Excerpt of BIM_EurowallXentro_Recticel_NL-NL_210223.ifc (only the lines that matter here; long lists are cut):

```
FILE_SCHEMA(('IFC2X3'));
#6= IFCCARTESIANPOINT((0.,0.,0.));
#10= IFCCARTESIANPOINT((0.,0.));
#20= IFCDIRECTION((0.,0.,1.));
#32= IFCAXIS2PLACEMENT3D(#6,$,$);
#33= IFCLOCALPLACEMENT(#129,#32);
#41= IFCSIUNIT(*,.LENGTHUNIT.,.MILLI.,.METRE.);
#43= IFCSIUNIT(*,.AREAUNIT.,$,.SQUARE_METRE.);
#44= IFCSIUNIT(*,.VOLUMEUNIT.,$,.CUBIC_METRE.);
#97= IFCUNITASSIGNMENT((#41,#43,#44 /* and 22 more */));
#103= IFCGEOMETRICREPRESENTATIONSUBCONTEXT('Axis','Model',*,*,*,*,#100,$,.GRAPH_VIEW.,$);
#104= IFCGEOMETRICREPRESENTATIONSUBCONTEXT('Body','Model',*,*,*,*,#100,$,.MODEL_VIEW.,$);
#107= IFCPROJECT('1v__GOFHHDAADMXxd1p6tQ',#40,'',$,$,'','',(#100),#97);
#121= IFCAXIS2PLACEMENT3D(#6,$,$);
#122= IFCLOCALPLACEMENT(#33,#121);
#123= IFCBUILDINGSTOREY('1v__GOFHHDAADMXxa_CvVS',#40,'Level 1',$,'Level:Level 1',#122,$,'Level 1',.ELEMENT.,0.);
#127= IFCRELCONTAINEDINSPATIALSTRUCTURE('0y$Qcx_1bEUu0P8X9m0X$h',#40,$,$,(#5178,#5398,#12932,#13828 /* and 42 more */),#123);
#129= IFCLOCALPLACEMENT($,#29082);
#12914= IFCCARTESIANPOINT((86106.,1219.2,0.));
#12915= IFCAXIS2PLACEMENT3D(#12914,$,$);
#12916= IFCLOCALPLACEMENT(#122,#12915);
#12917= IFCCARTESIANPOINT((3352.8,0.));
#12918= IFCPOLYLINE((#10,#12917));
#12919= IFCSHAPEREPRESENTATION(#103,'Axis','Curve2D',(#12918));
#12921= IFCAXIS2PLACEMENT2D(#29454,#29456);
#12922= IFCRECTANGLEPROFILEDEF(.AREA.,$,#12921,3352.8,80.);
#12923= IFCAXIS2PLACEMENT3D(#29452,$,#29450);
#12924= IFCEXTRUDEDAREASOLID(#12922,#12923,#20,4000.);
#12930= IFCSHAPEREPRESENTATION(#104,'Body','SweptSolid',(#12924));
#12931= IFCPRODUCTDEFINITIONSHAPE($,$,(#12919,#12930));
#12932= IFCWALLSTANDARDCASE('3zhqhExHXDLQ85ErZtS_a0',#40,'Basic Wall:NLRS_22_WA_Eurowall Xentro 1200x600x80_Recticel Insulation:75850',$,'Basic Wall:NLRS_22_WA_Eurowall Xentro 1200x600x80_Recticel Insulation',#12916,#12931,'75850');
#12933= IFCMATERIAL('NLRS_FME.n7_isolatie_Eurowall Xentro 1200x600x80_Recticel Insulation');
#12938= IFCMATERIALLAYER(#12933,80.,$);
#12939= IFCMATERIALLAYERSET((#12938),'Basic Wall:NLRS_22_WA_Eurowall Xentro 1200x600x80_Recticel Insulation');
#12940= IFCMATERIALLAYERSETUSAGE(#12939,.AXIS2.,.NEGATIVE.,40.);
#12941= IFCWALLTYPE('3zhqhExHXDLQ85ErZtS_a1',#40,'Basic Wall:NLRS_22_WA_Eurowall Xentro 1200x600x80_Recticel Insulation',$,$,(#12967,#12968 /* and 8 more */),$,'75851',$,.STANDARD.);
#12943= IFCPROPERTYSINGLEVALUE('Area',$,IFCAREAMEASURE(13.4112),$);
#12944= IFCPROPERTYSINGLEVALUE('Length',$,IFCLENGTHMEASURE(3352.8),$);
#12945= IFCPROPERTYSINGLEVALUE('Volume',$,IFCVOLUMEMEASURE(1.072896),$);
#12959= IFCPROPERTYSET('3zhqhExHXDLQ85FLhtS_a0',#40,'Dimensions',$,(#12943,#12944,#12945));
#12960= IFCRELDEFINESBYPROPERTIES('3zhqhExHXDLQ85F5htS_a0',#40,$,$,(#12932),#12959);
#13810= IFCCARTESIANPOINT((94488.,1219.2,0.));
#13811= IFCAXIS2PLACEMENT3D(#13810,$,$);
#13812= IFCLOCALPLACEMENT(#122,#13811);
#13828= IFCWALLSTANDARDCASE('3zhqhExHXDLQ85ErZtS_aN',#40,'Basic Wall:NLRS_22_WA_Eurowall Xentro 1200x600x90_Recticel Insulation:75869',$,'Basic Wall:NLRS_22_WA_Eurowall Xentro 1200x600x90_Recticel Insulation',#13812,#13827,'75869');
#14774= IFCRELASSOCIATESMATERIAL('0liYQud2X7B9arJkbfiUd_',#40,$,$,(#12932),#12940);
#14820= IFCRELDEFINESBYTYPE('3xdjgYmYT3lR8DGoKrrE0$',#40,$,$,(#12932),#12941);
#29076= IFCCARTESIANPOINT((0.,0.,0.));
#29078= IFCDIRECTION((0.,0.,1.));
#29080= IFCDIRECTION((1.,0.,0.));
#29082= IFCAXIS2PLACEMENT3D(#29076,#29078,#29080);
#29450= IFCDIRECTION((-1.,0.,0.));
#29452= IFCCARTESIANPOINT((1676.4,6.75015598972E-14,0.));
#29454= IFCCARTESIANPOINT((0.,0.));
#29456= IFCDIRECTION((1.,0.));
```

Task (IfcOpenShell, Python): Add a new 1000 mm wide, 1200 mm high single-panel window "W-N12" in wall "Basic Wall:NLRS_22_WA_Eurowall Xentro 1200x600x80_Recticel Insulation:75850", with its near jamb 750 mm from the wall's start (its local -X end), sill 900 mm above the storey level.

```python
import numpy as np
import ifcopenshell
import ifcopenshell.api.feature
import ifcopenshell.api.geometry
import ifcopenshell.api.pset
import ifcopenshell.api.root
import ifcopenshell.api.spatial
import ifcopenshell.api.type
import ifcopenshell.geom
import ifcopenshell.util.element
import ifcopenshell.util.placement
import ifcopenshell.util.representation
import ifcopenshell.util.shape
import ifcopenshell.util.unit

model = ifcopenshell.open("BIM_EurowallXentro_Recticel_NL-NL_210223.ifc")
unit_scale = ifcopenshell.util.unit.calculate_unit_scale(model)
area_scale = ifcopenshell.util.unit.calculate_unit_scale(model, "AREAUNIT")
volume_scale = ifcopenshell.util.unit.calculate_unit_scale(model, "VOLUMEUNIT")
settings = ifcopenshell.geom.settings()


def volume(element):
    """Net volume in cubic metres, openings subtracted."""
    shape = ifcopenshell.geom.create_shape(settings, element)
    return ifcopenshell.util.shape.get_volume(shape.geometry)


wall = model.by_guid("3zhqhExHXDLQ85ErZtS_a0")
storey = ifcopenshell.util.element.get_container(wall, ifc_class="IfcBuildingStorey")
context = ifcopenshell.util.representation.get_context(model, "Model", "Body", "MODEL_VIEW")
before = volume(wall)

width, height, from_end, sill = 1, 1.2, 0.75, 0.9  # metres

# The wall runs along its own X axis, and the end named is its -X end.
wall_shape = ifcopenshell.geom.create_shape(settings, wall)
x, y, z = ifcopenshell.util.shape.get_vertices(wall_shape.geometry).T
start = x.min() + from_end
face, thickness = float(y.min()), float(y.max() - y.min())
wall_matrix = ifcopenshell.util.placement.get_local_placement(wall.ObjectPlacement)
level = ifcopenshell.util.placement.get_local_placement(storey.ObjectPlacement)[2, 3]


def in_wall(x, y):
    """Placement at x, y metres in the wall's axes, at sill height."""
    matrix = wall_matrix.copy()
    matrix[:, 3] = wall_matrix @ np.array([x / unit_scale, y / unit_scale, 0.0, 1.0])
    matrix[2, 3] = level + sill / unit_scale
    return matrix


# Opening: a box that overshoots both wall faces by 50 mm.
opening = ifcopenshell.api.root.create_entity(model, ifc_class="IfcOpeningElement")
box = ifcopenshell.api.geometry.add_wall_representation(
    model, context=context, length=width, height=height, thickness=thickness + 0.1
)
ifcopenshell.api.geometry.assign_representation(model, product=opening, representation=box)
ifcopenshell.api.geometry.edit_object_placement(model, product=opening, matrix=in_wall(start, face - 0.05), is_si=False)
ifcopenshell.api.feature.add_feature(model, feature=opening, element=wall)

window = ifcopenshell.api.root.create_entity(model, ifc_class="IfcWindow", name="W-N12")
window.OverallWidth, window.OverallHeight = width / unit_scale, height / unit_scale
body = ifcopenshell.api.geometry.add_window_representation(
    model,
    context=context,
    overall_width=window.OverallWidth,
    overall_height=window.OverallHeight,
    partition_type="SINGLE_PANEL",
)
ifcopenshell.api.geometry.assign_representation(model, product=window, representation=body)
ifcopenshell.api.spatial.assign_container(model, products=[window], relating_structure=storey)
fills = ifcopenshell.api.feature.add_filling(model, opening=opening, element=window)
fills.OwnerHistory = window.OwnerHistory  # required in IFC2X3

# IFC2X3 keeps the operation on the window style.
style = ifcopenshell.api.root.create_entity(model, ifc_class="IfcWindowStyle", name="W-N12")
style.OperationType, style.ConstructionType = "SINGLE_PANEL", "NOTDEFINED"
style.ParameterTakesPrecedence = style.Sizeable = False
ifcopenshell.api.type.assign_type(model, related_objects=[window], relating_type=style)

# Centre the window in the wall's thickness.
ifcopenshell.api.geometry.edit_object_placement(model, product=window, matrix=in_wall(start, face), is_si=False)
window_shape = ifcopenshell.geom.create_shape(settings, window)
depth = ifcopenshell.util.shape.get_vertices(window_shape.geometry)[:, 1]
offset = face + thickness / 2 - (depth.min() + depth.max()) / 2
ifcopenshell.api.geometry.edit_object_placement(model, product=window, matrix=in_wall(start, offset), is_si=False)

after = volume(wall)

# Update the wall's stored quantities.
pset = model.by_id(ifcopenshell.util.element.get_pset(wall, "Dimensions", should_inherit=False)["id"])
ifcopenshell.api.pset.edit_pset(model, pset=pset, properties={
    "Area": model.create_entity("IfcAreaMeasure", after / thickness / area_scale),
    "Volume": model.create_entity("IfcVolumeMeasure", after / volume_scale),
})

print(f"wall volume {before:.3f} -> {after:.3f} m3")

model.write("BIM_EurowallXentro_Recticel_NL-NL_210223_v2.ifc")
```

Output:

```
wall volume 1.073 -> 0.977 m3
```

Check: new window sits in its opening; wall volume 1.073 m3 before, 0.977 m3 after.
